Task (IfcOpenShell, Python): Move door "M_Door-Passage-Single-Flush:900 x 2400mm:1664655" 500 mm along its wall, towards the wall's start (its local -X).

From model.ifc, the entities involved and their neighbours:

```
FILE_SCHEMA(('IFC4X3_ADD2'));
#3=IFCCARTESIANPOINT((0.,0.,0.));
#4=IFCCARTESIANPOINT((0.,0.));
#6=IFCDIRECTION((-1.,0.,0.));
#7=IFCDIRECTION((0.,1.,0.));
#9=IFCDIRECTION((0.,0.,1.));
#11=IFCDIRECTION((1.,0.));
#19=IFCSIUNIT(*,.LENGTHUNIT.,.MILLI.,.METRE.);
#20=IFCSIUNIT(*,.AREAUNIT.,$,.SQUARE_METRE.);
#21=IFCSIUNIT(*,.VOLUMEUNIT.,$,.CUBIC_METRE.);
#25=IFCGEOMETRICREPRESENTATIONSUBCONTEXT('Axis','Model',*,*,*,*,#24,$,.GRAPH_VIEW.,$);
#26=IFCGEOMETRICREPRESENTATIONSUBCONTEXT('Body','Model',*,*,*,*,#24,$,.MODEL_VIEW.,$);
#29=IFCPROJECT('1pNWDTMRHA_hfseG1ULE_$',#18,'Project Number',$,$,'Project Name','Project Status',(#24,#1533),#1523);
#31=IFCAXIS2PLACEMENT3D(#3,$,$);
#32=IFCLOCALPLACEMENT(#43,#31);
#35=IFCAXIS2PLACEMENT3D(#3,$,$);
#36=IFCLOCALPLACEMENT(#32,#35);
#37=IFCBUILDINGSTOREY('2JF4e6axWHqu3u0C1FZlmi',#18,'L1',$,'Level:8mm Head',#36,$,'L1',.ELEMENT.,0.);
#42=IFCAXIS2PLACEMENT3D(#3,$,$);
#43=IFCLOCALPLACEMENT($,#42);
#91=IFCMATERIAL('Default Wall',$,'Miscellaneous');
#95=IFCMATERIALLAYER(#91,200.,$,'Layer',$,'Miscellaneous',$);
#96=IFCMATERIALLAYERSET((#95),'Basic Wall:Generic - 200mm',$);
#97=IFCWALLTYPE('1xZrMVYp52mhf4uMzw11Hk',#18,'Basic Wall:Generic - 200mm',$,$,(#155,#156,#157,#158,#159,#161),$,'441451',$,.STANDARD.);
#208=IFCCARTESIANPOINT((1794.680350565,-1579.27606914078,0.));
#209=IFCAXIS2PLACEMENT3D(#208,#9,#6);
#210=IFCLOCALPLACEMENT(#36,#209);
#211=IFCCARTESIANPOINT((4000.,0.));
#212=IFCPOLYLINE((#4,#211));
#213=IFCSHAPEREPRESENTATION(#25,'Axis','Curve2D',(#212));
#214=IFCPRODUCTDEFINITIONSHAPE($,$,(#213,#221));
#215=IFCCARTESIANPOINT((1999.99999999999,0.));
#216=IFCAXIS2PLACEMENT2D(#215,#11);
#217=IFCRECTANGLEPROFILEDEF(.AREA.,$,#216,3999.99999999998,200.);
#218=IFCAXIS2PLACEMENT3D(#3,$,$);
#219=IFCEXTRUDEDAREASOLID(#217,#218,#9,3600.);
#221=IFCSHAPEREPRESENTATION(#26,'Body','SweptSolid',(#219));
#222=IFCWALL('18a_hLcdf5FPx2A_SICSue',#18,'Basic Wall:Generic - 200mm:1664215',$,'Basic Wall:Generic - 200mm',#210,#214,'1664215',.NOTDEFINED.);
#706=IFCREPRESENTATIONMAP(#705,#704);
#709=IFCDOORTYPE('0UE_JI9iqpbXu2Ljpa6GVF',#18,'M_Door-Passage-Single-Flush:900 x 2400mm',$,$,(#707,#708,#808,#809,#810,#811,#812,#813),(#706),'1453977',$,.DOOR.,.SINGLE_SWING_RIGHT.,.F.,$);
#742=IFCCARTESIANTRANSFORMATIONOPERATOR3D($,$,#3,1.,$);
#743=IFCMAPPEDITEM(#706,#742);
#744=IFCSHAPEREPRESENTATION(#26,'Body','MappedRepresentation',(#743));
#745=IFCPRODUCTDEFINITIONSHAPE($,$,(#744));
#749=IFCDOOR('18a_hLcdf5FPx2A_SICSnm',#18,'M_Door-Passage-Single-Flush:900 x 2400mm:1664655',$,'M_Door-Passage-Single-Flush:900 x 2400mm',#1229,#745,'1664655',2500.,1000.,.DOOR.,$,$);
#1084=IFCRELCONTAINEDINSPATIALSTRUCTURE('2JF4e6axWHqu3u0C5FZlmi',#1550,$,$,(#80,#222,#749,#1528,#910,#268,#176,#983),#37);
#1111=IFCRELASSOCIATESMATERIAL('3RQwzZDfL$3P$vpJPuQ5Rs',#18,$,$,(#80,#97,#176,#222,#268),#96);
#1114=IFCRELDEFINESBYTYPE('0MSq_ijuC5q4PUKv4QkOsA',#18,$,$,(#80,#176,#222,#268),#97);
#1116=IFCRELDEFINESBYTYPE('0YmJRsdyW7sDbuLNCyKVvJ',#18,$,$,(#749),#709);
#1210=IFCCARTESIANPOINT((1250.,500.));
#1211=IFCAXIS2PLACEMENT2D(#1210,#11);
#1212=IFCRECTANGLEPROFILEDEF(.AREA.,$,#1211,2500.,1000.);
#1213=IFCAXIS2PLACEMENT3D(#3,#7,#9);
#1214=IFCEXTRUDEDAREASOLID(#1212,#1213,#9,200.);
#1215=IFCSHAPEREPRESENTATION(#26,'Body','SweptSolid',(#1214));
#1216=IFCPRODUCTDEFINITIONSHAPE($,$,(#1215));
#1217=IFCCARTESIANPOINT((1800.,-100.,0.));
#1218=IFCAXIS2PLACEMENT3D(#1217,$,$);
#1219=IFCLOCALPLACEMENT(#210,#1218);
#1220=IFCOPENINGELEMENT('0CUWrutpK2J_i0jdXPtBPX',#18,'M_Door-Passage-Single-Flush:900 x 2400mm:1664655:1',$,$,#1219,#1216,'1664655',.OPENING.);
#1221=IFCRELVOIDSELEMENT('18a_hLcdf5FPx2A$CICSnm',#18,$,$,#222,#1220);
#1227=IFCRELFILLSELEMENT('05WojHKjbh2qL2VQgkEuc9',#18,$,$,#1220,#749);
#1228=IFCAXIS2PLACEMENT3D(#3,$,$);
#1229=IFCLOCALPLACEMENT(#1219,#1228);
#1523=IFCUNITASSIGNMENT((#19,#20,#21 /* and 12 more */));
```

```python
import ifcopenshell
import ifcopenshell.api.geometry
import ifcopenshell.util.placement
import ifcopenshell.util.unit

model = ifcopenshell.open("model.ifc")
unit_scale = ifcopenshell.util.unit.calculate_unit_scale(model)

door = model.by_id(749)
opening = door.FillsVoids[0].RelatingOpeningElement
wall = opening.VoidsElements[0].RelatingBuildingElement

wall_matrix = ifcopenshell.util.placement.get_local_placement(wall.ObjectPlacement)
shift = wall_matrix[:3, 0] * -0.5 / unit_scale
before = ifcopenshell.util.placement.get_local_placement(door.ObjectPlacement)[:3, 3].copy()

# The door is placed relative to its opening, so it follows when the opening moves.
matrix = ifcopenshell.util.placement.get_local_placement(opening.ObjectPlacement)
matrix[:3, 3] += shift
ifcopenshell.api.geometry.edit_object_placement(
    model, product=opening, matrix=matrix, is_si=False, should_transform_children=True
)

after = ifcopenshell.util.placement.get_local_placement(door.ObjectPlacement)[:3, 3]
print("door moved by", (after - before).round(3) + 0.0)

model.write("model-out.ifc")
```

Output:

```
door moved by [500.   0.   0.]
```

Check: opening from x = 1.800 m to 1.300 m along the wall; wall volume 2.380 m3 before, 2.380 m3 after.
